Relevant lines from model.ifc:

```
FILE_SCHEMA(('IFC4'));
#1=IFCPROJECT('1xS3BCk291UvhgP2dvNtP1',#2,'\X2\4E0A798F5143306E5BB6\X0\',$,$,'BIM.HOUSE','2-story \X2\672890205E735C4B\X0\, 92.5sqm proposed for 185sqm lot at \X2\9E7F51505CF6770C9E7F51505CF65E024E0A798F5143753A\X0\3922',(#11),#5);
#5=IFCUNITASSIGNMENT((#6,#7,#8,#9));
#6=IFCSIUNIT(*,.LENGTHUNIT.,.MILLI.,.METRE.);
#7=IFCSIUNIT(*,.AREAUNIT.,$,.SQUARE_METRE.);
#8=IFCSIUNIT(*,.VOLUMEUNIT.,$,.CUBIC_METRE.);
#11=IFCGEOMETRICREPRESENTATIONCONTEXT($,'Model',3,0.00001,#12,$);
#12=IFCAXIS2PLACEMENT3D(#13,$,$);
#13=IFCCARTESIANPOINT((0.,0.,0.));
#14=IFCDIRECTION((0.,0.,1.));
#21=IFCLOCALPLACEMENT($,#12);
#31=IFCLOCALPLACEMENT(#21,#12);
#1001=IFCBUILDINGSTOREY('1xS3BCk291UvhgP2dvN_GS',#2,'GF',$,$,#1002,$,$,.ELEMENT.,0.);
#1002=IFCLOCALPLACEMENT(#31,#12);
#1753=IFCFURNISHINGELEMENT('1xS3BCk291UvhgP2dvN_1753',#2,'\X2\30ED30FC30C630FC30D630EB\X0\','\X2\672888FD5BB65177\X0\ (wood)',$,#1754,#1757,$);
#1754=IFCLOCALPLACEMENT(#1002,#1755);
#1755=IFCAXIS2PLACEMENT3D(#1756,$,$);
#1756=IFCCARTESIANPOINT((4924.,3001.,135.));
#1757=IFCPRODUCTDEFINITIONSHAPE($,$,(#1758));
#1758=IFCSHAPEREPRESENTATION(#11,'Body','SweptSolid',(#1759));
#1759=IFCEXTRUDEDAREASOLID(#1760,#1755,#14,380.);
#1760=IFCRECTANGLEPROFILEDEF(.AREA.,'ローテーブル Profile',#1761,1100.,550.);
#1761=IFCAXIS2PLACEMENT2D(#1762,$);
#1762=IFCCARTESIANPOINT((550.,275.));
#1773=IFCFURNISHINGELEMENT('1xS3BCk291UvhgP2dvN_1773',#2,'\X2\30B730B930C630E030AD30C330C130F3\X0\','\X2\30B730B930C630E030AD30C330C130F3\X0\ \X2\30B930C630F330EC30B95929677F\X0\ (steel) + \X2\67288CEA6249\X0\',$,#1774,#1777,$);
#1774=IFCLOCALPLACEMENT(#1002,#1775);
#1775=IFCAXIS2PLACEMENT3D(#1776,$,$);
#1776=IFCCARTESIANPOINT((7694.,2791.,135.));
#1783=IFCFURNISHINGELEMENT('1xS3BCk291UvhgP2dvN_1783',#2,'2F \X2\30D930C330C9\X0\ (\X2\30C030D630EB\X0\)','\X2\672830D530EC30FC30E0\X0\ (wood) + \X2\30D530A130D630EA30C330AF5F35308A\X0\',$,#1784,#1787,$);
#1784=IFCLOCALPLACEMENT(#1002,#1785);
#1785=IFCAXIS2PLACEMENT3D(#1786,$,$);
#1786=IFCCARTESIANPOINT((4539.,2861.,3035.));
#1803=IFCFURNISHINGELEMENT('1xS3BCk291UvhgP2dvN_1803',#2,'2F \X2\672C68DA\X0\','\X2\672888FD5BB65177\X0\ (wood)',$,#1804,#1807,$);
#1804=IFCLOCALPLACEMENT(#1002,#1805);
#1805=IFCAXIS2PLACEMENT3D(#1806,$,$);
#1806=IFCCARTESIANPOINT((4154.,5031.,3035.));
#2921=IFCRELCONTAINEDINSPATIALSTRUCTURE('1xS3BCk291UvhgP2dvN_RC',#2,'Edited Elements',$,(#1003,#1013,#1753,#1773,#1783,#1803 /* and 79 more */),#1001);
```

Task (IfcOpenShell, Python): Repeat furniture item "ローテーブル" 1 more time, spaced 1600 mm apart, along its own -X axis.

```python
import ifcopenshell
import ifcopenshell.api.geometry
import ifcopenshell.api.root
import ifcopenshell.util.element
import ifcopenshell.util.placement

model = ifcopenshell.open("model.ifc")


def reuse_history(source, copy):
    """copy_class also copies each property set's owner history, people and application; keep the originals."""
    for rel in copy.IsDefinedBy:
        if rel.is_a("IfcRelDefinesByProperties") and (history := rel.RelatingPropertyDefinition.OwnerHistory):
            rel.RelatingPropertyDefinition.OwnerHistory = source.OwnerHistory
            ifcopenshell.util.element.remove_deep2(model, history)


source = model.by_id(1753)
base = ifcopenshell.util.placement.get_local_placement(source.ObjectPlacement)
step = -base[:3, 0] * 1600.0

for i in range(1, 2):
    copy = ifcopenshell.api.root.copy_class(model, product=source)
    copy.Representation = ifcopenshell.util.element.copy_deep(
        model, source.Representation, exclude=["IfcGeometricRepresentationContext", "IfcRepresentationMap"]
    )
    reuse_history(source, copy)
    matrix = base.copy()
    matrix[:3, 3] += i * step
    print("added at", matrix[:3, 3].round(3) + 0.0)
    ifcopenshell.api.geometry.edit_object_placement(model, product=copy, matrix=matrix, is_si=False)

model.write("model_v2.ifc")
```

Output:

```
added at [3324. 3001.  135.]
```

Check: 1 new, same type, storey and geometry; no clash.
